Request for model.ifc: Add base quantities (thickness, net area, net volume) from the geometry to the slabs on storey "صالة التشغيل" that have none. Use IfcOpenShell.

First a look at what the model holds.

```python
import ifcopenshell
import ifcopenshell.util.element
import ifcopenshell.util.unit

model = ifcopenshell.open("model.ifc")
print(model.schema)
for unit_type in ("LENGTHUNIT", "AREAUNIT", "VOLUMEUNIT"):
    print(unit_type, ifcopenshell.util.unit.calculate_unit_scale(model, unit_type))
storey = next(s for s in model.by_type("IfcBuildingStorey") if s.Name == "صالة التشغيل")
slabs = [e for e in ifcopenshell.util.element.get_decomposition(storey) if e.is_a("IfcSlab")]
for e in sorted(slabs, key=lambda e: e.id()):
    print(e.id(), e.is_a(), e.Name, list(ifcopenshell.util.element.get_psets(e, qtos_only=True)), sep=" | ")
```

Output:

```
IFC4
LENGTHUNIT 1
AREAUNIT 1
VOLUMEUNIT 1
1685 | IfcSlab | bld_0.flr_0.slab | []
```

```python
import ifcopenshell
import ifcopenshell.api.pset
import ifcopenshell.geom
import ifcopenshell.util.element
import ifcopenshell.util.shape
import ifcopenshell.util.unit

model = ifcopenshell.open("model.ifc")
unit_scale = ifcopenshell.util.unit.calculate_unit_scale(model)
area_scale = ifcopenshell.util.unit.calculate_unit_scale(model, "AREAUNIT")
volume_scale = ifcopenshell.util.unit.calculate_unit_scale(model, "VOLUMEUNIT")
settings = ifcopenshell.geom.settings()

storey = next(s for s in model.by_type("IfcBuildingStorey") if s.Name == "صالة التشغيل")
slabs = [e for e in ifcopenshell.util.element.get_decomposition(storey) if e.is_a("IfcSlab")]

for e in sorted(slabs, key=lambda e: e.id()):
    if ifcopenshell.util.element.get_psets(e, qtos_only=True, should_inherit=False):
        continue
    # Geometry comes back in metres, in the element's own axes.
    shape = ifcopenshell.geom.create_shape(settings, e)
    values = {
        "Width": ifcopenshell.util.shape.get_z(shape.geometry) / unit_scale,
        "NetArea": ifcopenshell.util.shape.get_footprint_area(shape.geometry) / area_scale,
        "NetVolume": ifcopenshell.util.shape.get_volume(shape.geometry) / volume_scale,
    }
    qto = ifcopenshell.api.pset.add_qto(model, product=e, name="Qto_SlabBaseQuantities")
    ifcopenshell.api.pset.edit_qto(model, qto=qto, properties=values)
    print(e.id(), {k: round(v, 3) for k, v in values.items()})

model.write("model_edited.ifc")
```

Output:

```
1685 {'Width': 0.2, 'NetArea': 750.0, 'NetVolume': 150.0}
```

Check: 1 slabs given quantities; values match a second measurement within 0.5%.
